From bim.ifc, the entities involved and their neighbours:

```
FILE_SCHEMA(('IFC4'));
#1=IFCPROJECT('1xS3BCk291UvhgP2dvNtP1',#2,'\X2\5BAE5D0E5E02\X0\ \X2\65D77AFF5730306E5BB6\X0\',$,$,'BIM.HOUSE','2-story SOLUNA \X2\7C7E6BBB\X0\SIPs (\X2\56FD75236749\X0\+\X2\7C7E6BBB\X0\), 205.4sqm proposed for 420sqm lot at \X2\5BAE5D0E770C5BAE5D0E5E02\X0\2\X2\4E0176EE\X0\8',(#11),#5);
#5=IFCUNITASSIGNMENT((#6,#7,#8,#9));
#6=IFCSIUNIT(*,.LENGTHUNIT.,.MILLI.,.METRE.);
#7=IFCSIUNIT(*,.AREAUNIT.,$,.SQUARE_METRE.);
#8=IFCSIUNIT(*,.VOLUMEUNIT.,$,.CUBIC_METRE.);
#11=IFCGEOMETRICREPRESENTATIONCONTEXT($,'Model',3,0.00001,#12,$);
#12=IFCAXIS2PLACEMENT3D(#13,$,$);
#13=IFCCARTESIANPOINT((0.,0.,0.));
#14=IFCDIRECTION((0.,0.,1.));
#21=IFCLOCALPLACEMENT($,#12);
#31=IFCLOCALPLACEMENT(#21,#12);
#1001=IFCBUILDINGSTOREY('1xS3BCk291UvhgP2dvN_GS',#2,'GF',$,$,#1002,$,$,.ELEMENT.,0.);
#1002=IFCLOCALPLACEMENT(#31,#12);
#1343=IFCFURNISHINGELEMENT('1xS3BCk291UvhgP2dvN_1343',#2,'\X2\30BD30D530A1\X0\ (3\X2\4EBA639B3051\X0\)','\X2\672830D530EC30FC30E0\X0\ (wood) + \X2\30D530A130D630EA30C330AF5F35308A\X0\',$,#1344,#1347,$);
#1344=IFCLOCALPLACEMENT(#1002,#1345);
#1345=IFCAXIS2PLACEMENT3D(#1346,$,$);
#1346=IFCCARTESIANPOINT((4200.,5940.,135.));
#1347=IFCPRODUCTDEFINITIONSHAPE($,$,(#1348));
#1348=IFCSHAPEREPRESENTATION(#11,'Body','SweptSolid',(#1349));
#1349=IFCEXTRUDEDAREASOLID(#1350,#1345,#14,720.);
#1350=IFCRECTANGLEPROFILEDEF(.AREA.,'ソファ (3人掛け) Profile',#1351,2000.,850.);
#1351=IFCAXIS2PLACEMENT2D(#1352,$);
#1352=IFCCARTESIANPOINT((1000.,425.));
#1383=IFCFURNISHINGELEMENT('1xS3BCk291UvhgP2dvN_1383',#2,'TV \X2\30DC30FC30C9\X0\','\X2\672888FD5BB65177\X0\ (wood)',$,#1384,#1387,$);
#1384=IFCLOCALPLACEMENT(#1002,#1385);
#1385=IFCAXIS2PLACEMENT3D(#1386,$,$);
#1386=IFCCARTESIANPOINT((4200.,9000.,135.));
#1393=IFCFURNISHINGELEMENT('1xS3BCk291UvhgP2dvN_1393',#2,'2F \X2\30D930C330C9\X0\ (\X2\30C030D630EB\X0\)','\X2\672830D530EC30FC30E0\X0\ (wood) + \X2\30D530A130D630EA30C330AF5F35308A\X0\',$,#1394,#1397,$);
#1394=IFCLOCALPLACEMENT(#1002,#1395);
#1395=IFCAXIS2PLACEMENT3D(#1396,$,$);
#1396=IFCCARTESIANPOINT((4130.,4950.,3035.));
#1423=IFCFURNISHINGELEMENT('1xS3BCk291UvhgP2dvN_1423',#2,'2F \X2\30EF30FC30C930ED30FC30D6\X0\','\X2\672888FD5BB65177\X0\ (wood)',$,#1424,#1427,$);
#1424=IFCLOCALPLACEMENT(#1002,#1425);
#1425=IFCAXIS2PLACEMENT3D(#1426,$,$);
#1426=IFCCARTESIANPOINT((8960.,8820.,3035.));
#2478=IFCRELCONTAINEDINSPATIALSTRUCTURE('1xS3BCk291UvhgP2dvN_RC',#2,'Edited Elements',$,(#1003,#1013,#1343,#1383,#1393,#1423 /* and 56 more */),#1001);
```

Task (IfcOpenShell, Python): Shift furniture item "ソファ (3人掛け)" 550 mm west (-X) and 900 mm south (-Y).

```python
import ifcopenshell
import ifcopenshell.api.geometry
import ifcopenshell.util.placement
import ifcopenshell.util.unit

model = ifcopenshell.open("bim.ifc")
unit_scale = ifcopenshell.util.unit.calculate_unit_scale(model)

item = model.by_id(1343)
matrix = ifcopenshell.util.placement.get_local_placement(item.ObjectPlacement)
matrix[0, 3] -= 0.55 / unit_scale
matrix[1, 3] -= 0.9 / unit_scale
ifcopenshell.api.geometry.edit_object_placement(model, product=item, matrix=matrix, is_si=False)

print(ifcopenshell.util.placement.get_local_placement(item.ObjectPlacement).round(3) + 0.0)

model.write("bim_rev.ifc")
```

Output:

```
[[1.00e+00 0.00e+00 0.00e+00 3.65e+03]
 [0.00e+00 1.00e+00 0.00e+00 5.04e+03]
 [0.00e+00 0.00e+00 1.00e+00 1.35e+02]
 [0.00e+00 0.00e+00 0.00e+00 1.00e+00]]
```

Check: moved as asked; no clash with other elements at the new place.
